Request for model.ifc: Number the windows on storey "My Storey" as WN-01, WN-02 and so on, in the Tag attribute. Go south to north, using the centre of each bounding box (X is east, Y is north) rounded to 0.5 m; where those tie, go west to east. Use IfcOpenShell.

First a look at what the model holds.

```python
import ifcopenshell
import ifcopenshell.util.element
import ifcopenshell.util.placement

model = ifcopenshell.open("model.ifc")
print(model.schema)
storey = next(s for s in model.by_type("IfcBuildingStorey") if s.Name == "My Storey")
windows = [e for e in ifcopenshell.util.element.get_decomposition(storey) if e.is_a("IfcWindow")]
for e in sorted(windows, key=lambda e: e.id()):
    origin = ifcopenshell.util.placement.get_local_placement(e.ObjectPlacement)[:3, 3]
    print(e.id(), e.Tag, e.Name, origin.round(2) + 0.0, sep=" | ")
```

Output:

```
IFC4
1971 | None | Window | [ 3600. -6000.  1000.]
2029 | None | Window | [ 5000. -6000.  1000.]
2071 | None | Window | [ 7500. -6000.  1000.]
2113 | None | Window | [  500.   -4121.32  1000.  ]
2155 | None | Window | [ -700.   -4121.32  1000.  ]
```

```python
import ifcopenshell
import ifcopenshell.geom
import ifcopenshell.util.element
import ifcopenshell.util.shape

model = ifcopenshell.open("model.ifc")
settings = ifcopenshell.geom.settings()
settings.set("use-world-coords", True)


def centre(element):
    shape = ifcopenshell.geom.create_shape(settings, element)
    return ifcopenshell.util.shape.get_bbox_centroid(shape.geometry)


storey = next(s for s in model.by_type("IfcBuildingStorey") if s.Name == "My Storey")
windows = [e for e in ifcopenshell.util.element.get_decomposition(storey) if e.is_a("IfcWindow")]

# Insertion points can sit at a corner or the storey origin, so sort by the geometry (in metres).
centres = {e: centre(e) for e in windows}
windows.sort(key=lambda e: (round(centres[e][1] / 0.5), centres[e][0]))

for i, e in enumerate(windows, start=1):
    number = f"WN-{i:02d}"
    e.Tag = number
    print(e.id(), number)

model.write("model_edited.ifc")
```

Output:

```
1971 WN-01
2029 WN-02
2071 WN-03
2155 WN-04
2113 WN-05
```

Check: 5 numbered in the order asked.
